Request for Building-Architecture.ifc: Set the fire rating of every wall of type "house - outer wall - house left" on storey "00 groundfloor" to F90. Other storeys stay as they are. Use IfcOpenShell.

First a look at what the model holds.

```python
import ifcopenshell
import ifcopenshell.util.element

model = ifcopenshell.open("Building-Architecture.ifc")
print(model.schema)
storey = next(s for s in model.by_type("IfcBuildingStorey") if s.Name == "00 groundfloor")
walls = [e for e in ifcopenshell.util.element.get_decomposition(storey) if e.is_a("IfcWall")]
seen = {}
for e in walls:
    element_type = ifcopenshell.util.element.get_type(e)
    key = (element_type.Name if element_type != e and element_type else None, ifcopenshell.util.element.get_pset(e, "Pset_WallCommon", "FireRating"))
    seen[key] = seen.get(key, 0) + 1
for (name, value), count in sorted(seen.items(), key=str):
    print(count, "x", name, "|", value)
```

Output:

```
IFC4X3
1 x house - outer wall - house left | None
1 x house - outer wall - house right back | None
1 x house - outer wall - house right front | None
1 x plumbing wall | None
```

```python
import ifcopenshell
import ifcopenshell.api.pset
import ifcopenshell.util.element

model = ifcopenshell.open("Building-Architecture.ifc")

storey = next(s for s in model.by_type("IfcBuildingStorey") if s.Name == "00 groundfloor")
walls = [e for e in ifcopenshell.util.element.get_decomposition(storey) if e.is_a("IfcWall")]

count = 0
for e in walls:
    element_type = ifcopenshell.util.element.get_type(e)
    if element_type in (None, e) or element_type.Name != "house - outer wall - house left":
        continue
    # add_pset returns the element's existing set when there is one.
    pset = ifcopenshell.api.pset.add_pset(model, product=e, name="Pset_WallCommon")
    ifcopenshell.api.pset.edit_pset(model, pset=pset, properties={"FireRating": "F90"})
    count += 1

print(count, "walls updated")

model.write("Building-Architecture-out.ifc")
```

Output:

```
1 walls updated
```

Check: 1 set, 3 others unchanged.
